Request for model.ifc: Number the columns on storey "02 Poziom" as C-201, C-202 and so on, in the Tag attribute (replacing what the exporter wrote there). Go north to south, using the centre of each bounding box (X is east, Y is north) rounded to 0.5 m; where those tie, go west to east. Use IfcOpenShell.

First a look at what the model holds.

```python
import ifcopenshell
import ifcopenshell.util.element
import ifcopenshell.util.placement

model = ifcopenshell.open("model.ifc")
print(model.schema)
storey = next(s for s in model.by_type("IfcBuildingStorey") if s.Name == "02 Poziom")
columns = [e for e in ifcopenshell.util.element.get_decomposition(storey) if e.is_a("IfcColumn")]
for e in sorted(columns, key=lambda e: e.id()):
    origin = ifcopenshell.util.placement.get_local_placement(e.ObjectPlacement)[:3, 3]
    print(e.id(), e.Tag, e.Name, origin.round(2) + 0.0, sep=" | ")
```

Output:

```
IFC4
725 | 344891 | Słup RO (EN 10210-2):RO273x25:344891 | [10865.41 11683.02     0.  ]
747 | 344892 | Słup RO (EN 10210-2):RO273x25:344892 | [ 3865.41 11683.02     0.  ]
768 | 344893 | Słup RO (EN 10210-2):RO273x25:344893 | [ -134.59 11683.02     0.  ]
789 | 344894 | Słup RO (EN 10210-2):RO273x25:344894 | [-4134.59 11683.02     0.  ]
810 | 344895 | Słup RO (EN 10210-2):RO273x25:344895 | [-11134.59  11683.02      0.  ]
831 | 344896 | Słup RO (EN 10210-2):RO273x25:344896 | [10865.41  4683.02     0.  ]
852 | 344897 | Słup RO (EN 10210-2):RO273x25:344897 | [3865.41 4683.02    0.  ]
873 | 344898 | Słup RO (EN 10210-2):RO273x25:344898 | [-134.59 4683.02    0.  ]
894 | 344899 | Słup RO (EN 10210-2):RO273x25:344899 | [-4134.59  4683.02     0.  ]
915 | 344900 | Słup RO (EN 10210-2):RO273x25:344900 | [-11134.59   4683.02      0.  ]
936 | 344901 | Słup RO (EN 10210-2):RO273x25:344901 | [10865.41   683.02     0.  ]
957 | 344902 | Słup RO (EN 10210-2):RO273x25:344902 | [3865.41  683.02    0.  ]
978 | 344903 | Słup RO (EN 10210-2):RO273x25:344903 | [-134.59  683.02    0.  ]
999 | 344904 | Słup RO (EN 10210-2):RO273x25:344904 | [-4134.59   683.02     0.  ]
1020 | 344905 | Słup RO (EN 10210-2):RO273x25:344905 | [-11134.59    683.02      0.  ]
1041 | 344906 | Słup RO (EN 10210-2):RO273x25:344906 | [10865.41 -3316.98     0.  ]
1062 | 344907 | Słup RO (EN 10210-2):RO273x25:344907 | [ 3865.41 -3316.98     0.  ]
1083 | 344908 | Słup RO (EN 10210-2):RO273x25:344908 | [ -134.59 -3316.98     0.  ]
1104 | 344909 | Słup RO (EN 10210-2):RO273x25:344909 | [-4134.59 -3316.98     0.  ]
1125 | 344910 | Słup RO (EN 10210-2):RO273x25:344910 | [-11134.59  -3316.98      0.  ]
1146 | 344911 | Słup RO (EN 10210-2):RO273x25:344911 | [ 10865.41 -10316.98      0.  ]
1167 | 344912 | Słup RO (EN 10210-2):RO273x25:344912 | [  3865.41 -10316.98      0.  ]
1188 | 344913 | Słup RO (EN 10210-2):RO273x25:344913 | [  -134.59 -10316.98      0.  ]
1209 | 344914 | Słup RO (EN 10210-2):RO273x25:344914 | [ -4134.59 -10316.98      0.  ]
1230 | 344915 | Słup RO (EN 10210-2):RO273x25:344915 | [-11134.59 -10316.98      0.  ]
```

```python
import ifcopenshell
import ifcopenshell.geom
import ifcopenshell.util.element
import ifcopenshell.util.shape

model = ifcopenshell.open("model.ifc")
settings = ifcopenshell.geom.settings()
settings.set("use-world-coords", True)


def centre(element):
    shape = ifcopenshell.geom.create_shape(settings, element)
    return ifcopenshell.util.shape.get_bbox_centroid(shape.geometry)


storey = next(s for s in model.by_type("IfcBuildingStorey") if s.Name == "02 Poziom")
columns = [e for e in ifcopenshell.util.element.get_decomposition(storey) if e.is_a("IfcColumn")]

# Insertion points can sit at a corner or the storey origin, so sort by the geometry (in metres).
centres = {e: centre(e) for e in columns}
columns.sort(key=lambda e: (-round(centres[e][1] / 0.5), centres[e][0]))

for i, e in enumerate(columns, start=1):
    number = f"C-2{i:02d}"
    e.Tag = number
    print(e.id(), number)

model.write("model-out.ifc")
```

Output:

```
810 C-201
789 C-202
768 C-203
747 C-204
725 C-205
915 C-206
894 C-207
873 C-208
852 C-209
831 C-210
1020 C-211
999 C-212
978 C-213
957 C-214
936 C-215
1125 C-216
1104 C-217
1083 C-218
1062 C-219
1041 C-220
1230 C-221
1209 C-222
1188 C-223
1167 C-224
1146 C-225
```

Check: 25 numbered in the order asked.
